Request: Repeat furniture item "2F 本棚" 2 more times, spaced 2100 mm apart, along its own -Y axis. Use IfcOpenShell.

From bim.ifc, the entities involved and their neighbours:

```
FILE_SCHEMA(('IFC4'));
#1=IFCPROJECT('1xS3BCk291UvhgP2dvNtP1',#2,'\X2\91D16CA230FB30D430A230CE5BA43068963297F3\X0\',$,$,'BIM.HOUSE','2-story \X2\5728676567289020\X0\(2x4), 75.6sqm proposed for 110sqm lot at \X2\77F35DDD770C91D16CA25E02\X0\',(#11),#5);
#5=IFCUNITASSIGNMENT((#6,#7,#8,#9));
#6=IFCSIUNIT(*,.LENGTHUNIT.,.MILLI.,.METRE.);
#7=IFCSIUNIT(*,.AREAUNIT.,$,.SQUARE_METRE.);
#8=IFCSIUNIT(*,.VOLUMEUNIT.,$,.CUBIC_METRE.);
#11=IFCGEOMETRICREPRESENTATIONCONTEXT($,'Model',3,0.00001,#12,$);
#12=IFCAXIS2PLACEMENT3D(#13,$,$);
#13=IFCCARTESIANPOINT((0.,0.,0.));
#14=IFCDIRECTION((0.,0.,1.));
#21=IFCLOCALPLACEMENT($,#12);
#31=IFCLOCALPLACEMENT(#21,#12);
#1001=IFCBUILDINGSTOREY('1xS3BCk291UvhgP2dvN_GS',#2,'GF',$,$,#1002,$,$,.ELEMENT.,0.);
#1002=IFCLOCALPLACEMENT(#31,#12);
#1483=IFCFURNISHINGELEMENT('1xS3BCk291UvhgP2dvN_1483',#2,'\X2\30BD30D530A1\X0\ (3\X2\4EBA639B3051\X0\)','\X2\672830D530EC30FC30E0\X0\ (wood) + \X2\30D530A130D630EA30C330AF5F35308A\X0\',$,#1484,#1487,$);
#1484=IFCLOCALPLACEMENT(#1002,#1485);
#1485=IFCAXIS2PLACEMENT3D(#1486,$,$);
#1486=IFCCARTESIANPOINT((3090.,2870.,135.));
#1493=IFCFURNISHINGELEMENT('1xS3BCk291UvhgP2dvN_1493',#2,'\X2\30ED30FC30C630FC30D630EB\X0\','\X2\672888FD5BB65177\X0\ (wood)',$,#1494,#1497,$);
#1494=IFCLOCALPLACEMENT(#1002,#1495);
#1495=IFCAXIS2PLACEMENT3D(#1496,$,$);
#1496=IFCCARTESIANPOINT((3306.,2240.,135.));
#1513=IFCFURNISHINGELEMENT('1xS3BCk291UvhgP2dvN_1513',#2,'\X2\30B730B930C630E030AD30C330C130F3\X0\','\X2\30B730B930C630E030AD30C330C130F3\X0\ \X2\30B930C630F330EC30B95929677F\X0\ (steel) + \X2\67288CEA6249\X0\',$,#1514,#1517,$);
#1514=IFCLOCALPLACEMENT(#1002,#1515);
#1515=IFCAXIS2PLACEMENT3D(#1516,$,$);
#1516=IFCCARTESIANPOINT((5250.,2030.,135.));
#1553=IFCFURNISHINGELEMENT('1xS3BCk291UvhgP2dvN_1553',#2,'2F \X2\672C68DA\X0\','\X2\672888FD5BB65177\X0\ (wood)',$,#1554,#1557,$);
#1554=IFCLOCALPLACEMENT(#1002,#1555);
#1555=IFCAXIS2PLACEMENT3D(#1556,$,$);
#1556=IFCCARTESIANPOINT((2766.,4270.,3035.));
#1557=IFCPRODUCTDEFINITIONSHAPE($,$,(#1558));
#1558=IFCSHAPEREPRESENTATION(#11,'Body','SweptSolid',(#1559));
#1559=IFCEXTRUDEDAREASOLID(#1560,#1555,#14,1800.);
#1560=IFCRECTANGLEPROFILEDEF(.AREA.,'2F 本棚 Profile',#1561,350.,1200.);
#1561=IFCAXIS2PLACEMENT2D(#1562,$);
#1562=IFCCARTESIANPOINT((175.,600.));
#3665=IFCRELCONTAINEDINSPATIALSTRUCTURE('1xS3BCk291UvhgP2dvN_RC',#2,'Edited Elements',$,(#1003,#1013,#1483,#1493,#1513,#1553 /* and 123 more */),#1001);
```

```python
import ifcopenshell
import ifcopenshell.api.geometry
import ifcopenshell.api.root
import ifcopenshell.util.element
import ifcopenshell.util.placement
import ifcopenshell.util.unit

model = ifcopenshell.open("bim.ifc")
unit_scale = ifcopenshell.util.unit.calculate_unit_scale(model)


def reuse_history(source, copy):
    """copy_class also copies each property set's owner history, people and application; keep the originals."""
    for rel in copy.IsDefinedBy:
        if rel.is_a("IfcRelDefinesByProperties") and (history := rel.RelatingPropertyDefinition.OwnerHistory):
            rel.RelatingPropertyDefinition.OwnerHistory = source.OwnerHistory
            ifcopenshell.util.element.remove_deep2(model, history)


source = model.by_guid("1xS3BCk291UvhgP2dvN_1553")
base = ifcopenshell.util.placement.get_local_placement(source.ObjectPlacement)
step = -base[:3, 1] * 2.1 / unit_scale

for i in range(1, 3):
    copy = ifcopenshell.api.root.copy_class(model, product=source)
    copy.Representation = ifcopenshell.util.element.copy_deep(
        model, source.Representation, exclude=["IfcGeometricRepresentationContext", "IfcRepresentationMap"]
    )
    reuse_history(source, copy)
    matrix = base.copy()
    matrix[:3, 3] += i * step
    print("added at", matrix[:3, 3].round(3) + 0.0)
    ifcopenshell.api.geometry.edit_object_placement(model, product=copy, matrix=matrix, is_si=False)

model.write("bim-out.ifc")
```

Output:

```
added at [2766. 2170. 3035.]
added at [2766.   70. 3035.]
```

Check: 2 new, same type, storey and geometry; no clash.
